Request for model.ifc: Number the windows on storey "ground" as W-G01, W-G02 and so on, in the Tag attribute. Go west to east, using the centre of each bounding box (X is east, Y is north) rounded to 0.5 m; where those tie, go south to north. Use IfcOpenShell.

First a look at what the model holds.

```python
import ifcopenshell
import ifcopenshell.util.element
import ifcopenshell.util.placement

model = ifcopenshell.open("model.ifc")
print(model.schema)
storey = next(s for s in model.by_type("IfcBuildingStorey") if s.Name == "ground")
windows = [e for e in ifcopenshell.util.element.get_decomposition(storey) if e.is_a("IfcWindow")]
for e in sorted(windows, key=lambda e: e.id()):
    origin = ifcopenshell.util.placement.get_local_placement(e.ObjectPlacement)[:3, 3]
    print(e.id(), e.Tag, e.Name, origin.round(2) + 0.0, sep=" | ")
```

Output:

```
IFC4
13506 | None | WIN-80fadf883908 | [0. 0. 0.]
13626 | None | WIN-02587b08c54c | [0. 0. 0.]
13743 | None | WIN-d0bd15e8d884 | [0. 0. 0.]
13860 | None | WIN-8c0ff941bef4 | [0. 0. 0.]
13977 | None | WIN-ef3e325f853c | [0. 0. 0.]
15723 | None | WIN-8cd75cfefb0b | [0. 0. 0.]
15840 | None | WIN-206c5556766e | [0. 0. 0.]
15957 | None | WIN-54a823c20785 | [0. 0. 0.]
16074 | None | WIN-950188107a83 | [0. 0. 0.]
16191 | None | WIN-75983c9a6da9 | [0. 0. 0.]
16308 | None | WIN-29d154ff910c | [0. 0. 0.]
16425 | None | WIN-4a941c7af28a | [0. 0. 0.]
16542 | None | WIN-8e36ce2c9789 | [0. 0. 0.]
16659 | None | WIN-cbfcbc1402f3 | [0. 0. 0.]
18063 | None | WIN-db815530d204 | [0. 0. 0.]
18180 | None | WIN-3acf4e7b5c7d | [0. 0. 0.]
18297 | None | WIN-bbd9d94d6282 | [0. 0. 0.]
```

```python
import ifcopenshell
import ifcopenshell.geom
import ifcopenshell.util.element
import ifcopenshell.util.shape

model = ifcopenshell.open("model.ifc")
settings = ifcopenshell.geom.settings()
settings.set("use-world-coords", True)


def centre(element):
    shape = ifcopenshell.geom.create_shape(settings, element)
    return ifcopenshell.util.shape.get_bbox_centroid(shape.geometry)


storey = next(s for s in model.by_type("IfcBuildingStorey") if s.Name == "ground")
windows = [e for e in ifcopenshell.util.element.get_decomposition(storey) if e.is_a("IfcWindow")]

# Insertion points can sit at a corner or the storey origin, so sort by the geometry (in metres).
centres = {e: centre(e) for e in windows}
windows.sort(key=lambda e: (round(centres[e][0] / 0.5), centres[e][1]))

for i, e in enumerate(windows, start=1):
    number = f"W-G{i:02d}"
    e.Tag = number
    print(e.id(), number)

model.write("model_updated.ifc")
```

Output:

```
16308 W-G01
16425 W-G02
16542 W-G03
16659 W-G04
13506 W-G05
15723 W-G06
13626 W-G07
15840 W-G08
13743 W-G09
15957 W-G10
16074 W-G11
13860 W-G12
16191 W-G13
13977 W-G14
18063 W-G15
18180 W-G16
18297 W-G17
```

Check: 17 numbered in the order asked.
